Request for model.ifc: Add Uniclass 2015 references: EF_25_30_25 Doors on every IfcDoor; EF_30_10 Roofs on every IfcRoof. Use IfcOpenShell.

First a look at what the model holds.

```python
import ifcopenshell

model = ifcopenshell.open("model.ifc")
print(model.schema)
print("classifications:", [c.Name for c in model.by_type("IfcClassification")])
for ifc_class in ("IfcDoor", "IfcRoof", "IfcStair", "IfcWall", "IfcWindow"):
    print(ifc_class, len(model.by_type(ifc_class)))
```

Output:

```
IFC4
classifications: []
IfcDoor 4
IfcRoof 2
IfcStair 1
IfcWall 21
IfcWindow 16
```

```python
import ifcopenshell
import ifcopenshell.api.classification

model = ifcopenshell.open("model.ifc")

system = ifcopenshell.api.classification.add_classification(model, classification="Uniclass 2015")

codes = {
    "IfcDoor": ("EF_25_30_25", "Doors"),
    "IfcRoof": ("EF_30_10", "Roofs"),
}
for ifc_class, (code, name) in codes.items():
    products = model.by_type(ifc_class)
    ifcopenshell.api.classification.add_reference(
        model, products=products, classification=system, identification=code, name=name
    )
    print(code, len(products))

model.write("model_v2.ifc")
```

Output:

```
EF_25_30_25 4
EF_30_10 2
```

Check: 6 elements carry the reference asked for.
